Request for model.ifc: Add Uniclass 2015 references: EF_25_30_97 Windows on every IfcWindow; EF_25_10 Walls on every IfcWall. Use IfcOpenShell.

First a look at what the model holds.

```python
import ifcopenshell

model = ifcopenshell.open("model.ifc")
print(model.schema)
print("classifications:", [c.Name for c in model.by_type("IfcClassification")])
for ifc_class in ("IfcDoor", "IfcRoof", "IfcStair", "IfcWall", "IfcWindow"):
    print(ifc_class, len(model.by_type(ifc_class)))
```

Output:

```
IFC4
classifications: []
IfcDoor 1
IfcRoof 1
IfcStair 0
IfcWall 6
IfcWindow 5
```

```python
import ifcopenshell
import ifcopenshell.api.classification

model = ifcopenshell.open("model.ifc")

system = ifcopenshell.api.classification.add_classification(model, classification="Uniclass 2015")

codes = {
    "IfcWindow": ("EF_25_30_97", "Windows"),
    "IfcWall": ("EF_25_10", "Walls"),
}
for ifc_class, (code, name) in codes.items():
    products = model.by_type(ifc_class)
    ifcopenshell.api.classification.add_reference(
        model, products=products, classification=system, identification=code, name=name
    )
    print(code, len(products))

model.write("model_rev.ifc")
```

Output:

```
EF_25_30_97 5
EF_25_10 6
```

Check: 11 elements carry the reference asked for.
